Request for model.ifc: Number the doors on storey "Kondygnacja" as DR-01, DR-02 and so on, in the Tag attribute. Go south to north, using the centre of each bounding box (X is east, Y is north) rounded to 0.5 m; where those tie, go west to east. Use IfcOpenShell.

First a look at what the model holds.

```python
import ifcopenshell
import ifcopenshell.util.element
import ifcopenshell.util.placement

model = ifcopenshell.open("model.ifc")
print(model.schema)
storey = next(s for s in model.by_type("IfcBuildingStorey") if s.Name == "Kondygnacja")
doors = [e for e in ifcopenshell.util.element.get_decomposition(storey) if e.is_a("IfcDoor")]
for e in sorted(doors, key=lambda e: e.id()):
    origin = ifcopenshell.util.placement.get_local_placement(e.ObjectPlacement)[:3, 3]
    print(e.id(), e.Tag, e.Name, origin.round(2) + 0.0, sep=" | ")
```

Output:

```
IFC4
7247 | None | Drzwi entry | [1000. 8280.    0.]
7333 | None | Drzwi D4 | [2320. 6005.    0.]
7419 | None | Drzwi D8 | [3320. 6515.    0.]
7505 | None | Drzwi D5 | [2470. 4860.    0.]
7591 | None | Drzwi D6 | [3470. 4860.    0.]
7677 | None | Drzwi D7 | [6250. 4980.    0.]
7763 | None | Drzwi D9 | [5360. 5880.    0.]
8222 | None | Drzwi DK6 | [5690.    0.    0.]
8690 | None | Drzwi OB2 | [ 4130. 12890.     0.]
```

```python
import ifcopenshell
import ifcopenshell.geom
import ifcopenshell.util.element
import ifcopenshell.util.shape

model = ifcopenshell.open("model.ifc")
settings = ifcopenshell.geom.settings()
settings.set("use-world-coords", True)


def centre(element):
    shape = ifcopenshell.geom.create_shape(settings, element)
    return ifcopenshell.util.shape.get_bbox_centroid(shape.geometry)


storey = next(s for s in model.by_type("IfcBuildingStorey") if s.Name == "Kondygnacja")
doors = [e for e in ifcopenshell.util.element.get_decomposition(storey) if e.is_a("IfcDoor")]

# Insertion points can sit at a corner or the storey origin, so sort by the geometry (in metres).
centres = {e: centre(e) for e in doors}
doors.sort(key=lambda e: (round(centres[e][1] / 0.5), centres[e][0]))

for i, e in enumerate(doors, start=1):
    number = f"DR-{i:02d}"
    e.Tag = number
    print(e.id(), number)

model.write("model_edited.ifc")
```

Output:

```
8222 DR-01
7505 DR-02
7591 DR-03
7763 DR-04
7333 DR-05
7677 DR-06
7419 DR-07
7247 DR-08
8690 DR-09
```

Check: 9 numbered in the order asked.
